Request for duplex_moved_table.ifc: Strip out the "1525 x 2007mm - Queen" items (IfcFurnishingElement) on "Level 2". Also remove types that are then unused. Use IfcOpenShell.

First a look at what the model holds.

```python
import ifcopenshell
import ifcopenshell.util.element

model = ifcopenshell.open("duplex_moved_table.ifc")
print(model.schema)
storey = next(s for s in model.by_type("IfcBuildingStorey") if s.Name == "Level 2")
furniture = [e for e in ifcopenshell.util.element.get_decomposition(storey) if e.is_a("IfcFurnishingElement")]
seen = {}
for e in furniture:
    element_type = ifcopenshell.util.element.get_type(e)
    name = element_type.Name if element_type not in (None, e) else None
    seen[name] = seen.get(name, 0) + 1
for name, count in sorted(seen.items(), key=str):
    print(count, "x", name)
```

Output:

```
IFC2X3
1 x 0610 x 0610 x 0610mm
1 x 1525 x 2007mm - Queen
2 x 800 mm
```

```python
import ifcopenshell
import ifcopenshell.api.root
import ifcopenshell.util.element

model = ifcopenshell.open("duplex_moved_table.ifc")

storey = next(s for s in model.by_type("IfcBuildingStorey") if s.Name == "Level 2")
furniture = [e for e in ifcopenshell.util.element.get_decomposition(storey) if e.is_a("IfcFurnishingElement")]
targets = [e for e in furniture if (t := ifcopenshell.util.element.get_type(e)) not in (None, e) and t.Name == "1525 x 2007mm - Queen"]
types = {ifcopenshell.util.element.get_type(e) for e in targets} - {None, *targets}

for e in targets:
    ifcopenshell.api.root.remove_product(model, product=e)
print(len(targets), "removed")

unused = [t for t in types if not ifcopenshell.util.element.get_types(t)]
for t in unused:
    ifcopenshell.api.root.remove_product(model, product=t)
print(len(unused), "unused types removed")

model.write("duplex_moved_table_updated.ifc")
```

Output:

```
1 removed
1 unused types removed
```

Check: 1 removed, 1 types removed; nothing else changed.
